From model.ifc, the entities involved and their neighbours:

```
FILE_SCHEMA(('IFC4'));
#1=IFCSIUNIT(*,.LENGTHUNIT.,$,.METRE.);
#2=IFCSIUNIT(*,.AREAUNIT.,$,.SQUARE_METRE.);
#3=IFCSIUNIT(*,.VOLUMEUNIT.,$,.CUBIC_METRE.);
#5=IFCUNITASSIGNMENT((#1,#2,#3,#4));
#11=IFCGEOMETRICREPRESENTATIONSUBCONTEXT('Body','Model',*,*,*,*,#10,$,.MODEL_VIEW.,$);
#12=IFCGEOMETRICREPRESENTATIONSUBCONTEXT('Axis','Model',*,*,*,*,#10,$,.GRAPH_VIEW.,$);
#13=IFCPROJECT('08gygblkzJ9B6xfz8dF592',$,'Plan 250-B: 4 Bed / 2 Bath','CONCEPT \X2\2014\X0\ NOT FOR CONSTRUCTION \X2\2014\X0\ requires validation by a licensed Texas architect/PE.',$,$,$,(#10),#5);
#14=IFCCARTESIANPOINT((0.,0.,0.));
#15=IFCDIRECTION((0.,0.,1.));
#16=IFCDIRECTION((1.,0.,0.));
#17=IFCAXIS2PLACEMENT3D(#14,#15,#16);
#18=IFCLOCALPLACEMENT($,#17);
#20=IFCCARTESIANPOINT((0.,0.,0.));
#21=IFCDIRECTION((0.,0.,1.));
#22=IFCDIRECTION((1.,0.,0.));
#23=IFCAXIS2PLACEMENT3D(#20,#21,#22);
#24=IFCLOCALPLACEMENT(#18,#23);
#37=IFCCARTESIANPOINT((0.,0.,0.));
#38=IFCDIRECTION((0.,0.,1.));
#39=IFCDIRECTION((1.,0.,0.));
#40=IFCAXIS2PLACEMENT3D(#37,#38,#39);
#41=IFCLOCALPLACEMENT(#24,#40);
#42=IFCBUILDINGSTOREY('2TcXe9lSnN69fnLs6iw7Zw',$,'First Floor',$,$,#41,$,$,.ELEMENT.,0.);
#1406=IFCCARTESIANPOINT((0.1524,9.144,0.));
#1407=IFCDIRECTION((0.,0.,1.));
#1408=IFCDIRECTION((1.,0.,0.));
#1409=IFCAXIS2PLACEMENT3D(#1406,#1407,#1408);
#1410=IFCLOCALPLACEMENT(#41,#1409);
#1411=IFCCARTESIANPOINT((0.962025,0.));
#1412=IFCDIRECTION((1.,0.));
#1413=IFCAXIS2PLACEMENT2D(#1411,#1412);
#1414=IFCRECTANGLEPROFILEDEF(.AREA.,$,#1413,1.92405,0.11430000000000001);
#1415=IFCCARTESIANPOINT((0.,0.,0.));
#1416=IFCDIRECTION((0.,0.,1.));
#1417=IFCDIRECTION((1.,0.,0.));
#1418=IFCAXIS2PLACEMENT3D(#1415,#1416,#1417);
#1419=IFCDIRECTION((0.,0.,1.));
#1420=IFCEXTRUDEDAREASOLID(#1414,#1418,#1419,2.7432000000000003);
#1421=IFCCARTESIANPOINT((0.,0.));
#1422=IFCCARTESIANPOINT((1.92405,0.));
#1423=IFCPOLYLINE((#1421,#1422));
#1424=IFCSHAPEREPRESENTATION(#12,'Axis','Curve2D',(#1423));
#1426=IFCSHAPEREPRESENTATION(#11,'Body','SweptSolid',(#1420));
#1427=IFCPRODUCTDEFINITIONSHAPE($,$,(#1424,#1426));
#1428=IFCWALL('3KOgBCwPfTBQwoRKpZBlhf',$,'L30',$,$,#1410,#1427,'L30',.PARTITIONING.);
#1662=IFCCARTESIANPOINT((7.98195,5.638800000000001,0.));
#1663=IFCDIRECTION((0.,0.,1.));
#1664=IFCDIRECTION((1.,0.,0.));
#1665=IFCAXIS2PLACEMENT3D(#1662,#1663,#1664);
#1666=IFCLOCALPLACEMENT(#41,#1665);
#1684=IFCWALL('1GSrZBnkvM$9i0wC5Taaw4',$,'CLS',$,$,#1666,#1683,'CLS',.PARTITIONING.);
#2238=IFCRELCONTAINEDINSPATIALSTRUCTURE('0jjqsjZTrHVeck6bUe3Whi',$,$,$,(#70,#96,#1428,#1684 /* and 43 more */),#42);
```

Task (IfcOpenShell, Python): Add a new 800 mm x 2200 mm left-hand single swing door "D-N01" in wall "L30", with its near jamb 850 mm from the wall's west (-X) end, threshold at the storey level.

```python
import numpy as np
import ifcopenshell
import ifcopenshell.api.feature
import ifcopenshell.api.geometry
import ifcopenshell.api.root
import ifcopenshell.api.spatial
import ifcopenshell.geom
import ifcopenshell.util.element
import ifcopenshell.util.placement
import ifcopenshell.util.representation
import ifcopenshell.util.shape
import ifcopenshell.util.unit

model = ifcopenshell.open("model.ifc")
unit_scale = ifcopenshell.util.unit.calculate_unit_scale(model)
settings = ifcopenshell.geom.settings()


def volume(element):
    """Net volume in cubic metres, openings subtracted."""
    shape = ifcopenshell.geom.create_shape(settings, element)
    return ifcopenshell.util.shape.get_volume(shape.geometry)


wall = model.by_guid("3KOgBCwPfTBQwoRKpZBlhf")
storey = ifcopenshell.util.element.get_container(wall, ifc_class="IfcBuildingStorey")
context = ifcopenshell.util.representation.get_context(model, "Model", "Body", "MODEL_VIEW")
before = volume(wall)

width, height, from_end, sill = 0.8, 2.2, 0.85, 0.0  # metres

# The wall runs along its own X axis, and the end named is its -X end.
wall_shape = ifcopenshell.geom.create_shape(settings, wall)
x, y, z = ifcopenshell.util.shape.get_vertices(wall_shape.geometry).T
start = x.min() + from_end
face, thickness = float(y.min()), float(y.max() - y.min())
wall_matrix = ifcopenshell.util.placement.get_local_placement(wall.ObjectPlacement)
level = ifcopenshell.util.placement.get_local_placement(storey.ObjectPlacement)[2, 3]


def in_wall(x, y):
    """Placement at x, y metres in the wall's axes, at sill height."""
    matrix = wall_matrix.copy()
    matrix[:, 3] = wall_matrix @ np.array([x / unit_scale, y / unit_scale, 0.0, 1.0])
    matrix[2, 3] = level + sill / unit_scale
    return matrix


# Opening: a box that overshoots both wall faces by 50 mm.
opening = ifcopenshell.api.root.create_entity(model, ifc_class="IfcOpeningElement", predefined_type="OPENING")
box = ifcopenshell.api.geometry.add_wall_representation(
    model, context=context, length=width, height=height, thickness=thickness + 0.1
)
ifcopenshell.api.geometry.assign_representation(model, product=opening, representation=box)
ifcopenshell.api.geometry.edit_object_placement(model, product=opening, matrix=in_wall(start, face - 0.05), is_si=False)
ifcopenshell.api.feature.add_feature(model, feature=opening, element=wall)

door = ifcopenshell.api.root.create_entity(model, ifc_class="IfcDoor", name="D-N01", predefined_type="DOOR")
door.OverallWidth, door.OverallHeight = width / unit_scale, height / unit_scale
door.OperationType = "SINGLE_SWING_LEFT"
body = ifcopenshell.api.geometry.add_door_representation(
    model,
    context=context,
    overall_width=door.OverallWidth,
    overall_height=door.OverallHeight,
    operation_type="SINGLE_SWING_LEFT",
    lining_properties={"LiningDepth": thickness / unit_scale, "ThresholdDepth": thickness / unit_scale},
)
ifcopenshell.api.geometry.assign_representation(model, product=door, representation=body)
ifcopenshell.api.spatial.assign_container(model, products=[door], relating_structure=storey)
ifcopenshell.api.feature.add_filling(model, opening=opening, element=door)

# The lining spans the wall, so the door starts at the wall face.
ifcopenshell.api.geometry.edit_object_placement(model, product=door, matrix=in_wall(start, face), is_si=False)

after = volume(wall)

print(f"wall volume {before:.3f} -> {after:.3f} m3")

model.write("model_v2.ifc")
```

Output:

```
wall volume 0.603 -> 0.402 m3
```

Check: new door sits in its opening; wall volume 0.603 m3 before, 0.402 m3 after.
